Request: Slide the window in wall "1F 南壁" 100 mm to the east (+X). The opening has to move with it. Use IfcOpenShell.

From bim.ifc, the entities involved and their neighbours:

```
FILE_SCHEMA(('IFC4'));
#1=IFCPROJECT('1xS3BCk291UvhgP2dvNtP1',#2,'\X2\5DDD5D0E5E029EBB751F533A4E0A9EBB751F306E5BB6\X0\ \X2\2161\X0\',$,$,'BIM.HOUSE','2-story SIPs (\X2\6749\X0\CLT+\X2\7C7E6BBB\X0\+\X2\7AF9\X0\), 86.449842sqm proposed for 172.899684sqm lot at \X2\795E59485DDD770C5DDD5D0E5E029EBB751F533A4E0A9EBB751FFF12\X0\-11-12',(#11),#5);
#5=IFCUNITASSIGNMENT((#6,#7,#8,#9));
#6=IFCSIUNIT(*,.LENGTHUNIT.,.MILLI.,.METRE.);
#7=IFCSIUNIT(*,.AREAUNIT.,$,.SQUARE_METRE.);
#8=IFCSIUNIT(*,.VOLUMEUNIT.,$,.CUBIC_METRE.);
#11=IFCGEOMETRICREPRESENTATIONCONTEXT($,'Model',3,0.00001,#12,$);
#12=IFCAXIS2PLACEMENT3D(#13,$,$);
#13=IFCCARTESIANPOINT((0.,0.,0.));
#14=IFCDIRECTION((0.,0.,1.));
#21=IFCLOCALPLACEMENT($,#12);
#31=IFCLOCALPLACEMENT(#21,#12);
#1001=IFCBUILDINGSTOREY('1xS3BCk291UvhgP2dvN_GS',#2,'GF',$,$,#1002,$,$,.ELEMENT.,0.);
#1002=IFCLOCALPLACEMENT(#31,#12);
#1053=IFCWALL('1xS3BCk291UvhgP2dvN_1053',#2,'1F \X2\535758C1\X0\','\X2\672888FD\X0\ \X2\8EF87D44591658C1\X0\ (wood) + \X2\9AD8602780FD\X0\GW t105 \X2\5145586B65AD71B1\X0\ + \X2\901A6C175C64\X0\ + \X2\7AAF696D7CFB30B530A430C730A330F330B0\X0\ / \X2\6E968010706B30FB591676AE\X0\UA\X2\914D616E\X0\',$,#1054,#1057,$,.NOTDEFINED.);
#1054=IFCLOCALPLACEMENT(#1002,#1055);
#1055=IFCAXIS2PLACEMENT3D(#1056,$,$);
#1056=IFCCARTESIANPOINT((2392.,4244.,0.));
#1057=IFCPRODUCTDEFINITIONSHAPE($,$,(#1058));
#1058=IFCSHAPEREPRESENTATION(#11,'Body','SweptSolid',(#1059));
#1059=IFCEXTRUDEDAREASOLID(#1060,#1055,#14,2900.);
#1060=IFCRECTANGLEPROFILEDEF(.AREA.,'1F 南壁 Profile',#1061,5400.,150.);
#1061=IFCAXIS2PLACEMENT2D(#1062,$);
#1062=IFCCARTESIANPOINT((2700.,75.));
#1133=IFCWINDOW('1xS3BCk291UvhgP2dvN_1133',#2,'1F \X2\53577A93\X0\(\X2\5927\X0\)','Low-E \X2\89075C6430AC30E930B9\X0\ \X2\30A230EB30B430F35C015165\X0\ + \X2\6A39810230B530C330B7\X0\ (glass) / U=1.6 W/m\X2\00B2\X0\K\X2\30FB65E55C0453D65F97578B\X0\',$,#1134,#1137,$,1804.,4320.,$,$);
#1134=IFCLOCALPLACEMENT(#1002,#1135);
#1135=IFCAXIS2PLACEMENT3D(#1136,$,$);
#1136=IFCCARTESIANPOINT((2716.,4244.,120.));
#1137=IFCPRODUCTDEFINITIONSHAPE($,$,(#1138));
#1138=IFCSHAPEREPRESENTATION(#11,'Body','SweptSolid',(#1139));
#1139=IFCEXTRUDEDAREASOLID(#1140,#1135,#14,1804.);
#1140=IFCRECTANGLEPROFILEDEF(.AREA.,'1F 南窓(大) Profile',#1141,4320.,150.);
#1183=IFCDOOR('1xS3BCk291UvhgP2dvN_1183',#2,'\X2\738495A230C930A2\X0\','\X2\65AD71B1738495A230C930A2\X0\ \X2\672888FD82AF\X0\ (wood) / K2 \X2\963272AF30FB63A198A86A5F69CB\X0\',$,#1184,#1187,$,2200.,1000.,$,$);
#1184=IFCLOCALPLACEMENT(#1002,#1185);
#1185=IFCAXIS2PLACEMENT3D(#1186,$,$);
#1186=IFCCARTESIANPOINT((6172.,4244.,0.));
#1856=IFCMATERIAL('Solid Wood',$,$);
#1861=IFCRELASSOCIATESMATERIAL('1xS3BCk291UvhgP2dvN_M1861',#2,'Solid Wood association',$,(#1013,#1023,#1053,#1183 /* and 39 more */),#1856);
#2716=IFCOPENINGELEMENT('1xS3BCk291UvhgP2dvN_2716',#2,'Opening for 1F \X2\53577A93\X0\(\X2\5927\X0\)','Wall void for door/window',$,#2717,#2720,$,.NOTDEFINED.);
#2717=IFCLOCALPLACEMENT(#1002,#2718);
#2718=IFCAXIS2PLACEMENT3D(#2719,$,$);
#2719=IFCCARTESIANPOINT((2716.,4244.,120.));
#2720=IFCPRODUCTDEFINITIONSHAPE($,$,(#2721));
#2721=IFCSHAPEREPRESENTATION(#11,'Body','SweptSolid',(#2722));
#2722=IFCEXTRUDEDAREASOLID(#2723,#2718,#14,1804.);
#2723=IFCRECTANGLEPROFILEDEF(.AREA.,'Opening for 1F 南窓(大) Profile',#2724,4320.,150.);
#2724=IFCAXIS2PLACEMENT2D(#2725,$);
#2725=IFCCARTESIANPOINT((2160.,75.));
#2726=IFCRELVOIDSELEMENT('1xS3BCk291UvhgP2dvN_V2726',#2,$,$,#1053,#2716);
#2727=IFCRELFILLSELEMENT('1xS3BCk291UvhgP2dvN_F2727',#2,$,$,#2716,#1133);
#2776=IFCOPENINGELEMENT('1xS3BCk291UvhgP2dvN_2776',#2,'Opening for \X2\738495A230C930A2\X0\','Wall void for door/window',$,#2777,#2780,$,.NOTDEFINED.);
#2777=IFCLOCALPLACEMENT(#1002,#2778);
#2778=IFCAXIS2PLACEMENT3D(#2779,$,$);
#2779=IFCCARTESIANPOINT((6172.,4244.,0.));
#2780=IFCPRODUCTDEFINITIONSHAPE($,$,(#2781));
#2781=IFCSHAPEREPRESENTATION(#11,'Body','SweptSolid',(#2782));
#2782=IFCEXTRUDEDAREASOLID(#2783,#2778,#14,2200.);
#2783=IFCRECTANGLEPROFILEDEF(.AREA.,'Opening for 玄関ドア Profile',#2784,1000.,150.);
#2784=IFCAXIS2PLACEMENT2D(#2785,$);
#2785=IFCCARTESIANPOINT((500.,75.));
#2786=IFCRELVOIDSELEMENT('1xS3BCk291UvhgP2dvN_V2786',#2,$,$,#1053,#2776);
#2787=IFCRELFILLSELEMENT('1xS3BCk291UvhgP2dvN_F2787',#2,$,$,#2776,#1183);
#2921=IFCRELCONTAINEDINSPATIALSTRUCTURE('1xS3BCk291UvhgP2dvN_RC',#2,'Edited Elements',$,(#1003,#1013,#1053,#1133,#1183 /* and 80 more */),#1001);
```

```python
import ifcopenshell
import ifcopenshell.api.geometry
import ifcopenshell.util.placement
import ifcopenshell.util.unit

model = ifcopenshell.open("bim.ifc")
unit_scale = ifcopenshell.util.unit.calculate_unit_scale(model)

window = model.by_guid("1xS3BCk291UvhgP2dvN_1133")
opening = window.FillsVoids[0].RelatingOpeningElement
wall = opening.VoidsElements[0].RelatingBuildingElement

wall_matrix = ifcopenshell.util.placement.get_local_placement(wall.ObjectPlacement)
shift = wall_matrix[:3, 0] * 0.1 / unit_scale
before = ifcopenshell.util.placement.get_local_placement(window.ObjectPlacement)[:3, 3].copy()

# The window is not placed relative to its opening, so move both.
for product in (opening, window):
    matrix = ifcopenshell.util.placement.get_local_placement(product.ObjectPlacement)
    matrix[:3, 3] += shift
    ifcopenshell.api.geometry.edit_object_placement(model, product=product, matrix=matrix, is_si=False)

after = ifcopenshell.util.placement.get_local_placement(window.ObjectPlacement)[:3, 3]
print("window moved by", (after - before).round(3) + 0.0)

model.write("bim_updated.ifc")
```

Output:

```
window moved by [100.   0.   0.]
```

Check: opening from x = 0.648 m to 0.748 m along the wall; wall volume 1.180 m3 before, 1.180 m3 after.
